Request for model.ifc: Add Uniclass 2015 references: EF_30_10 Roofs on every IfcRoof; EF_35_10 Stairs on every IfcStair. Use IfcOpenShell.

First a look at what the model holds.

```python
import ifcopenshell

model = ifcopenshell.open("model.ifc")
print(model.schema)
print("classifications:", [c.Name for c in model.by_type("IfcClassification")])
for ifc_class in ("IfcDoor", "IfcRoof", "IfcStair", "IfcWall", "IfcWindow"):
    print(ifc_class, len(model.by_type(ifc_class)))
```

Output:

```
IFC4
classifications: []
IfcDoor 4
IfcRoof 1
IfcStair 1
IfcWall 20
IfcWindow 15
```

```python
import ifcopenshell
import ifcopenshell.api.classification

model = ifcopenshell.open("model.ifc")

system = ifcopenshell.api.classification.add_classification(model, classification="Uniclass 2015")

codes = {
    "IfcRoof": ("EF_30_10", "Roofs"),
    "IfcStair": ("EF_35_10", "Stairs"),
}
for ifc_class, (code, name) in codes.items():
    products = model.by_type(ifc_class)
    ifcopenshell.api.classification.add_reference(
        model, products=products, classification=system, identification=code, name=name
    )
    print(code, len(products))

model.write("model_edited.ifc")
```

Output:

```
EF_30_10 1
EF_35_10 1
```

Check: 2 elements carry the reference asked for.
